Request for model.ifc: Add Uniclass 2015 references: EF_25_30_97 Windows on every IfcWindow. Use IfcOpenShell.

First a look at what the model holds.

```python
import ifcopenshell

model = ifcopenshell.open("model.ifc")
print(model.schema)
print("classifications:", [c.Name for c in model.by_type("IfcClassification")])
for ifc_class in ("IfcDoor", "IfcRoof", "IfcStair", "IfcWall", "IfcWindow"):
    print(ifc_class, len(model.by_type(ifc_class)))
```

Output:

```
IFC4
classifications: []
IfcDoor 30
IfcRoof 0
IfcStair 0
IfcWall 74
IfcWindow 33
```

```python
import ifcopenshell
import ifcopenshell.api.classification

model = ifcopenshell.open("model.ifc")

system = ifcopenshell.api.classification.add_classification(model, classification="Uniclass 2015")

codes = {
    "IfcWindow": ("EF_25_30_97", "Windows"),
}
for ifc_class, (code, name) in codes.items():
    products = model.by_type(ifc_class)
    ifcopenshell.api.classification.add_reference(
        model, products=products, classification=system, identification=code, name=name
    )
    print(code, len(products))

model.write("model_edited.ifc")
```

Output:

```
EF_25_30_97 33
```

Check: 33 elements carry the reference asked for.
